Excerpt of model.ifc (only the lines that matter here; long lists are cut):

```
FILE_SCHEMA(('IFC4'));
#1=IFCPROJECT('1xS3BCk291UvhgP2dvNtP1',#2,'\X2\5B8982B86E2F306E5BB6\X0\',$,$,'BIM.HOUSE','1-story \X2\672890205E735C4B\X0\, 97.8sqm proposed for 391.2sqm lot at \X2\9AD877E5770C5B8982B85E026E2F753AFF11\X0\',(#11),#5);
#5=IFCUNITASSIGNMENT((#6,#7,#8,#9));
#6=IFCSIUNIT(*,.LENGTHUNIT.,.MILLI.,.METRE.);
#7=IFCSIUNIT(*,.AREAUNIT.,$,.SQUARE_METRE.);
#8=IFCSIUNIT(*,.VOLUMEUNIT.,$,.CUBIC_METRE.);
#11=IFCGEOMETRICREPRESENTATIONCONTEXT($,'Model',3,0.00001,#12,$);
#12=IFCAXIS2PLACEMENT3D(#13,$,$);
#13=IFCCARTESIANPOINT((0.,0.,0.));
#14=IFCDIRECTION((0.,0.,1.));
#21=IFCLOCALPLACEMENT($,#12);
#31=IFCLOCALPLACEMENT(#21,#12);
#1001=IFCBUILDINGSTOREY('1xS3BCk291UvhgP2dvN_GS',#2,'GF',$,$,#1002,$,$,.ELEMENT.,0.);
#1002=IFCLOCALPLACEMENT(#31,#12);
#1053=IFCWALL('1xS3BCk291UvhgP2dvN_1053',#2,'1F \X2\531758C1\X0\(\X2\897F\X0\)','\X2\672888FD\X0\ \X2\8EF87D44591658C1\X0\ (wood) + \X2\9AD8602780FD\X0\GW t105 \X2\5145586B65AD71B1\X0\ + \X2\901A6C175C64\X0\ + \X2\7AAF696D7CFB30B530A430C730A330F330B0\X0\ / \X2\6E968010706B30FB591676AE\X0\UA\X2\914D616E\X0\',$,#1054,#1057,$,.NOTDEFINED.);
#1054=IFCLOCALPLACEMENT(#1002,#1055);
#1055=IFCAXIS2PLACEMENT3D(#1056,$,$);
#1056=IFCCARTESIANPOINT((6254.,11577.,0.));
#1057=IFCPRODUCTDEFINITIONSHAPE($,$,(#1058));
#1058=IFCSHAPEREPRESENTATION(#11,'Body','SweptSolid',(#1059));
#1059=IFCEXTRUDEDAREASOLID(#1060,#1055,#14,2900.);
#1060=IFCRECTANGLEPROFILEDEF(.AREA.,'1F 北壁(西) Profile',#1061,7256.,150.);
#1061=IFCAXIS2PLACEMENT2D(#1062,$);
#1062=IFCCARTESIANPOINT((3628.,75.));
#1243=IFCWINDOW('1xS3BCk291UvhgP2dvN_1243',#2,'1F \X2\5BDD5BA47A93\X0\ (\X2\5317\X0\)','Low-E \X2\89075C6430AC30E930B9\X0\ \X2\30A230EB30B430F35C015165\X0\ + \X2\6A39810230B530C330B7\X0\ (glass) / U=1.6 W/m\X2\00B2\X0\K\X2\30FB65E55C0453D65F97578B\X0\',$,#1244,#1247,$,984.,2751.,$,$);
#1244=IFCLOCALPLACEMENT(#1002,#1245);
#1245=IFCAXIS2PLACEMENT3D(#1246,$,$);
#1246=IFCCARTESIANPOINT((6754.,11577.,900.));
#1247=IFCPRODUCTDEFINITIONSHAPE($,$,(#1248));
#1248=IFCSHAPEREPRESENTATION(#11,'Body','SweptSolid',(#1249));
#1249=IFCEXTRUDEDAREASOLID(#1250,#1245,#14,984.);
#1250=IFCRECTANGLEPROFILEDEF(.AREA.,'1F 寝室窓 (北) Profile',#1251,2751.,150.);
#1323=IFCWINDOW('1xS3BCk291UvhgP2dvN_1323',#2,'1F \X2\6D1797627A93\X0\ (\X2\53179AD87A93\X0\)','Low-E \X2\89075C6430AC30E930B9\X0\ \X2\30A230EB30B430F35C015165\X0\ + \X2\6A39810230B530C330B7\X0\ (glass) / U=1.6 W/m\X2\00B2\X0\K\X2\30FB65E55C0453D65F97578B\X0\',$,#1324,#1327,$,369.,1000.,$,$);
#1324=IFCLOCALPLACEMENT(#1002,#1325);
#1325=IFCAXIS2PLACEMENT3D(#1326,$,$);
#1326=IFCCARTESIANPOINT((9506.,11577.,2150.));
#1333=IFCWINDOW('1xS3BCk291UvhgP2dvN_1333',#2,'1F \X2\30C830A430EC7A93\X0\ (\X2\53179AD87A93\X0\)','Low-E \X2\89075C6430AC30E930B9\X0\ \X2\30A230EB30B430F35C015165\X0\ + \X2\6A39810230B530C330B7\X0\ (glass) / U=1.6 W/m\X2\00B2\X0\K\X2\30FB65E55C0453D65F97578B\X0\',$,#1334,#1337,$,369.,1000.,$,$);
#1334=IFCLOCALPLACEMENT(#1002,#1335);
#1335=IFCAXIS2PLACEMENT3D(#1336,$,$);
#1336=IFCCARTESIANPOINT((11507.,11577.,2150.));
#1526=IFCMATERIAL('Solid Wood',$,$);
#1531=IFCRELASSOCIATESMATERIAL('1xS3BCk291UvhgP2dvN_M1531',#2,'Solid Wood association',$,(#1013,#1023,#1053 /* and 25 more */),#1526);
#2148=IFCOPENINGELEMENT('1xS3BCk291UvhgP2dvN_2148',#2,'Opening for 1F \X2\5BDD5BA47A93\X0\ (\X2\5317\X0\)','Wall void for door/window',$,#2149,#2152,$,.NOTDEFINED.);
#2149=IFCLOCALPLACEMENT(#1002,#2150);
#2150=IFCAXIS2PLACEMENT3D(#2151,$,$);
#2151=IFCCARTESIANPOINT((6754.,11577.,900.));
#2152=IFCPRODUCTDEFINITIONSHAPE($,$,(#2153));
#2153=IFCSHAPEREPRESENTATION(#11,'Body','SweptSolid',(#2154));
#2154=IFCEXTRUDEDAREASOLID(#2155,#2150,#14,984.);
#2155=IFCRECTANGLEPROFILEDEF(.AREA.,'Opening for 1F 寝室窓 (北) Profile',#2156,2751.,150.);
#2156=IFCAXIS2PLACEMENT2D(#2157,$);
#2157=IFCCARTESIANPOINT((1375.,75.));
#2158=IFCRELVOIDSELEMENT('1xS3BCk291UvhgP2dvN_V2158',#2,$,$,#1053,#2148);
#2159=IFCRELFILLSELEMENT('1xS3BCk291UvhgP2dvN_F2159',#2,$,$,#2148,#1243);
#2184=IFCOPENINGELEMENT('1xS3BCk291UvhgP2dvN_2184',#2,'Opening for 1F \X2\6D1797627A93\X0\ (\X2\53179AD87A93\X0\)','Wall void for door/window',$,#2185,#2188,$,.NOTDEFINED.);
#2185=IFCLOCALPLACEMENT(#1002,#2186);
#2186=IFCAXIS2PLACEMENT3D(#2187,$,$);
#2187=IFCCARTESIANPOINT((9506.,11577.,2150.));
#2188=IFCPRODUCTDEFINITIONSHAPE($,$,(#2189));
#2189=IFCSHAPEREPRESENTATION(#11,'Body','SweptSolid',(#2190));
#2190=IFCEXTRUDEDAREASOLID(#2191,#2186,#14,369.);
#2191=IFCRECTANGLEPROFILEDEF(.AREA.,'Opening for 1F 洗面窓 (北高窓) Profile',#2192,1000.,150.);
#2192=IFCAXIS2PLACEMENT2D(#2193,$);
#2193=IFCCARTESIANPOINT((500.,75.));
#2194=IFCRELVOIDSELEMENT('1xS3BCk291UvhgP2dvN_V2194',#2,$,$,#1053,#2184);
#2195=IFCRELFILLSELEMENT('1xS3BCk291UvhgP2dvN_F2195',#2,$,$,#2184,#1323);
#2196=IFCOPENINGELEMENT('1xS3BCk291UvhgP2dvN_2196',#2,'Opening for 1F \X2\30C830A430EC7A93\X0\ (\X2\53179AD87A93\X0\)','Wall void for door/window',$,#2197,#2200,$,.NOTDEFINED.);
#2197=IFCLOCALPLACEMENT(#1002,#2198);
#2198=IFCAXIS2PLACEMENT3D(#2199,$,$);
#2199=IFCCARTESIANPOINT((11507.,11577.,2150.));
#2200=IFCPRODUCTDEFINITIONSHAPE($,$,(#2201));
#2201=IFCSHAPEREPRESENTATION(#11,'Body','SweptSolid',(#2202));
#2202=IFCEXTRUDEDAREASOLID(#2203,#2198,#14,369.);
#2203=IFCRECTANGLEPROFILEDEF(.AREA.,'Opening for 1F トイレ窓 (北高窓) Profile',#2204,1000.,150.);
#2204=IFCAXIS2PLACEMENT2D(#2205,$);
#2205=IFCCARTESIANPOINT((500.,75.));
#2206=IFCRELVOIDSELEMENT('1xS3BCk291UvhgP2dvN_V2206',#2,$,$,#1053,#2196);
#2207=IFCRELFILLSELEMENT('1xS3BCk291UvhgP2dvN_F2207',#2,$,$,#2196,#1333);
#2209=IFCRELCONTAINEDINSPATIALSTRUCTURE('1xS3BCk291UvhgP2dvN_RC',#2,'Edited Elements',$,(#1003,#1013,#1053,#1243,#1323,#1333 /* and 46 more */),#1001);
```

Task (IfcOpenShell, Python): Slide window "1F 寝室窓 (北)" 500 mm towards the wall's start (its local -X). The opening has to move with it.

```python
import ifcopenshell
import ifcopenshell.api.geometry
import ifcopenshell.util.placement
import ifcopenshell.util.unit

model = ifcopenshell.open("model.ifc")
unit_scale = ifcopenshell.util.unit.calculate_unit_scale(model)

window = model.by_id(1243)
opening = window.FillsVoids[0].RelatingOpeningElement
wall = opening.VoidsElements[0].RelatingBuildingElement

wall_matrix = ifcopenshell.util.placement.get_local_placement(wall.ObjectPlacement)
shift = wall_matrix[:3, 0] * -0.5 / unit_scale
before = ifcopenshell.util.placement.get_local_placement(window.ObjectPlacement)[:3, 3].copy()

# The window is not placed relative to its opening, so move both.
for product in (opening, window):
    matrix = ifcopenshell.util.placement.get_local_placement(product.ObjectPlacement)
    matrix[:3, 3] += shift
    ifcopenshell.api.geometry.edit_object_placement(model, product=product, matrix=matrix, is_si=False)

after = ifcopenshell.util.placement.get_local_placement(window.ObjectPlacement)[:3, 3]
print("window moved by", (after - before).round(3) + 0.0)

model.write("model_updated.ifc")
```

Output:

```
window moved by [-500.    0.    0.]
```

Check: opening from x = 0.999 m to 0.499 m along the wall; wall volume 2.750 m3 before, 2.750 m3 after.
